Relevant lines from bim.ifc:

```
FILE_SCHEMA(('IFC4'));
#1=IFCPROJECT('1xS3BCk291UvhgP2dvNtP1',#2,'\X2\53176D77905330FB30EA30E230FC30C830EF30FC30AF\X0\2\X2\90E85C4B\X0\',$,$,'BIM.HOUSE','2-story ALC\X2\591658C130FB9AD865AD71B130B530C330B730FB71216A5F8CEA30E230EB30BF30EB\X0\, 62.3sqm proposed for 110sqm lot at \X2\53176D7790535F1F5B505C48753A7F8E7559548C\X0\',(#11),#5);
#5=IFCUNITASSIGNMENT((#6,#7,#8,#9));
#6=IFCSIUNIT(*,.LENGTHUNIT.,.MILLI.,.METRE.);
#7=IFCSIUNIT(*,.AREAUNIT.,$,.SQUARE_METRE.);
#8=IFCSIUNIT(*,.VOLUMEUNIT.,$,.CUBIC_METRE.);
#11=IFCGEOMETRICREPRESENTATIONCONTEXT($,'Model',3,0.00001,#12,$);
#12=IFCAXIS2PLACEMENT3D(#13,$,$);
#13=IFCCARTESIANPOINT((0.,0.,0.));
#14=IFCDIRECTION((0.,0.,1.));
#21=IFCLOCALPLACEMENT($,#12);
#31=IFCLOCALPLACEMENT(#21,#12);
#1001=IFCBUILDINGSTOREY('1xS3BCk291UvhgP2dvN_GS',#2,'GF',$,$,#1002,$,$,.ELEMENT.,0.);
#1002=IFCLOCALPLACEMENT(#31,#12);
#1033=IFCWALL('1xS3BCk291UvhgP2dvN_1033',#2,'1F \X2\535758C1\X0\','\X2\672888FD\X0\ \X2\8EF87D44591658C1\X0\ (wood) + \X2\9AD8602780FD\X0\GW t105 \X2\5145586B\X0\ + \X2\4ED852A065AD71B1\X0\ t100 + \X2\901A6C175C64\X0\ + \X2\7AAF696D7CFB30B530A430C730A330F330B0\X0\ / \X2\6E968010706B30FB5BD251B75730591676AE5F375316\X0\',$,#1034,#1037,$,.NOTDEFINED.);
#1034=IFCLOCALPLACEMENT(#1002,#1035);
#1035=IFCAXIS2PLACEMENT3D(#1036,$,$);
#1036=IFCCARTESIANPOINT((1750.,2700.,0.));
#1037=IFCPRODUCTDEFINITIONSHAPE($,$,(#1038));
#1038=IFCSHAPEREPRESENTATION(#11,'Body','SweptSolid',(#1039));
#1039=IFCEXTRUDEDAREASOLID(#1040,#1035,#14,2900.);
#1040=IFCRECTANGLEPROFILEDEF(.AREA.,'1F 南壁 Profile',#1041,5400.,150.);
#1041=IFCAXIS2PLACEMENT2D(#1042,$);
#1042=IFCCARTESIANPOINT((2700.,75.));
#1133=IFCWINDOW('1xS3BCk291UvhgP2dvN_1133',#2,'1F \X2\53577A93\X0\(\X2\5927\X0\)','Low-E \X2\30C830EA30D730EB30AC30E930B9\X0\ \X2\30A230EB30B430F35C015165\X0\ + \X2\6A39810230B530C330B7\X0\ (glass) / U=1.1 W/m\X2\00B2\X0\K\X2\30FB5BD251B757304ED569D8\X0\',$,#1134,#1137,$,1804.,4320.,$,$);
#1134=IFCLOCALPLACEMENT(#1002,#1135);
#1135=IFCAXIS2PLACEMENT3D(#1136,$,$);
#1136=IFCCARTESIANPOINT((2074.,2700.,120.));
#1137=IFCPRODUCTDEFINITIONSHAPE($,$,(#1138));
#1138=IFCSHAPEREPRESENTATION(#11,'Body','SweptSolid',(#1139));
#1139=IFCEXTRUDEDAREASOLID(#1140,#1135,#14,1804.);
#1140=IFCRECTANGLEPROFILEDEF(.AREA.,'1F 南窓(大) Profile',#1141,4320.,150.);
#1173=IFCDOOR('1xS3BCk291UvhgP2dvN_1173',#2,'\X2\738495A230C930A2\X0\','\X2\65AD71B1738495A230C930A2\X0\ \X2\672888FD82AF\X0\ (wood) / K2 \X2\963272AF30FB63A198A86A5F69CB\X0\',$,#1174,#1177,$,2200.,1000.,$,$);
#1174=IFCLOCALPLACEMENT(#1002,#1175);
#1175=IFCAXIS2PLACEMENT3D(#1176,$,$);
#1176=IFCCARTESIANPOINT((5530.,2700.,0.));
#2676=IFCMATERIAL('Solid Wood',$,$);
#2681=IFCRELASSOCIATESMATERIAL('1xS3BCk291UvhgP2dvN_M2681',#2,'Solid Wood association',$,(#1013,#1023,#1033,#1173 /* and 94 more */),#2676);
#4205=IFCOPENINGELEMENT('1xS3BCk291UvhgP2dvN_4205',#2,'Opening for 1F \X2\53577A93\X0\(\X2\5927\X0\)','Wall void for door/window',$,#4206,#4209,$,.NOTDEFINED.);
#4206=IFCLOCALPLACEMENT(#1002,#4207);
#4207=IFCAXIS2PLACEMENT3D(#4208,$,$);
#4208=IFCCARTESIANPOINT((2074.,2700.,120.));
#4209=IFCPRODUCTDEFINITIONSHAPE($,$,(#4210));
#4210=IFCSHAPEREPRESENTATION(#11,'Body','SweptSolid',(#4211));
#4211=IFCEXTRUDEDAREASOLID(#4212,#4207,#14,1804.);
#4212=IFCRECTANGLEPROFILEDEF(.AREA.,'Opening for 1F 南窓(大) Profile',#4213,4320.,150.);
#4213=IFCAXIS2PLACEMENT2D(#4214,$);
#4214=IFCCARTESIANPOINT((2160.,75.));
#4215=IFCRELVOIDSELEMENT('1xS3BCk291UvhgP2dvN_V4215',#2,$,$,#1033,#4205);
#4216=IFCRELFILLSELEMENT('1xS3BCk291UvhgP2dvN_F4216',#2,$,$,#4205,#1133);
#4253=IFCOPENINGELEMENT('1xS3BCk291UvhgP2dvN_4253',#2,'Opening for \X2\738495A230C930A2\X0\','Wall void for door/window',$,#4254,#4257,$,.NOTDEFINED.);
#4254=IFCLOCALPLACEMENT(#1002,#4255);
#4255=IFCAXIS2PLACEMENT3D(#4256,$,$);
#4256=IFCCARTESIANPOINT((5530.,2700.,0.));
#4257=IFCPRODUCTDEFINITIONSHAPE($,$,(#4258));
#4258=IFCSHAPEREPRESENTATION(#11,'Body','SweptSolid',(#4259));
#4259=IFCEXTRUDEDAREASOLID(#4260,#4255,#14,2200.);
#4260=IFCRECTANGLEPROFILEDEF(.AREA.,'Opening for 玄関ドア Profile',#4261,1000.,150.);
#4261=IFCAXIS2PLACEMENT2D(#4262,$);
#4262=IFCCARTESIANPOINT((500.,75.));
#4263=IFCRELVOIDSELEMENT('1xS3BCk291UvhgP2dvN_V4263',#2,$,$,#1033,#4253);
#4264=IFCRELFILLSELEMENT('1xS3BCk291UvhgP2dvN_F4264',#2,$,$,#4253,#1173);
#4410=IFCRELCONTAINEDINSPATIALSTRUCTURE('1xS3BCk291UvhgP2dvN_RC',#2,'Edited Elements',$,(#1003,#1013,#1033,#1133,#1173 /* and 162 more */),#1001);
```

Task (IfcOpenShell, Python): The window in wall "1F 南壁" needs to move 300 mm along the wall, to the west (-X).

```python
import ifcopenshell
import ifcopenshell.api.geometry
import ifcopenshell.util.placement

model = ifcopenshell.open("bim.ifc")

window = model.by_id(1133)
opening = window.FillsVoids[0].RelatingOpeningElement
wall = opening.VoidsElements[0].RelatingBuildingElement

wall_matrix = ifcopenshell.util.placement.get_local_placement(wall.ObjectPlacement)
shift = wall_matrix[:3, 0] * -300.0
before = ifcopenshell.util.placement.get_local_placement(window.ObjectPlacement)[:3, 3].copy()

# The window is not placed relative to its opening, so move both.
for product in (opening, window):
    matrix = ifcopenshell.util.placement.get_local_placement(product.ObjectPlacement)
    matrix[:3, 3] += shift
    ifcopenshell.api.geometry.edit_object_placement(model, product=product, matrix=matrix, is_si=False)

after = ifcopenshell.util.placement.get_local_placement(window.ObjectPlacement)[:3, 3]
print("window moved by", (after - before).round(3) + 0.0)

model.write("bim_rev.ifc")
```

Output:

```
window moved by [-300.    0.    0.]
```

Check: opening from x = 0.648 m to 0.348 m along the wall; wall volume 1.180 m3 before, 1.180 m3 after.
